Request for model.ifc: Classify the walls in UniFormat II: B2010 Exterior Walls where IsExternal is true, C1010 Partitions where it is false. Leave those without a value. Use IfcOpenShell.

First a look at what the model holds.

```python
import ifcopenshell
import ifcopenshell.util.element

model = ifcopenshell.open("model.ifc")
print(model.schema)
print("classifications:", [c.Name for c in model.by_type("IfcClassification")])
values = [ifcopenshell.util.element.get_pset(e, "Pset_WallCommon", "IsExternal") for e in model.by_type("IfcWall")]
for value in (True, False, None):
    print("IsExternal", value, values.count(value))
```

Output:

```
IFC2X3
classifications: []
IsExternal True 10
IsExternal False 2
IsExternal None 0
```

```python
import ifcopenshell
import ifcopenshell.api.classification
import ifcopenshell.util.element

model = ifcopenshell.open("model.ifc")

# IFC2X3 requires Source and Edition and has no link from the project to the system.
system = model.create_entity("IfcClassification", Source="ASTM", Edition="E1557", Name="UniFormat II")

walls = model.by_type("IfcWall")
external = {e: ifcopenshell.util.element.get_pset(e, "Pset_WallCommon", "IsExternal") for e in walls}
for flag, code, name in ((True, "B2010", "Exterior Walls"), (False, "C1010", "Partitions")):
    products = [e for e in walls if external[e] is flag]
    ifcopenshell.api.classification.add_reference(
        model, products=products, classification=system, identification=code, name=name
    )
    print(code, len(products))

model.write("model_v2.ifc")
```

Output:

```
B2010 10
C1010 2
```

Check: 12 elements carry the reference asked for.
